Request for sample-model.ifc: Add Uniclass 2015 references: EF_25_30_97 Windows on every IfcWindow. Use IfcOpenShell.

First a look at what the model holds.

```python
import ifcopenshell

model = ifcopenshell.open("sample-model.ifc")
print(model.schema)
print("classifications:", [c.Name for c in model.by_type("IfcClassification")])
for ifc_class in ("IfcDoor", "IfcRoof", "IfcStair", "IfcWall", "IfcWindow"):
    print(ifc_class, len(model.by_type(ifc_class)))
```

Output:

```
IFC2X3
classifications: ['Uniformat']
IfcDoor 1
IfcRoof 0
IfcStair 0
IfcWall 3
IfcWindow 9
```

```python
import ifcopenshell
import ifcopenshell.api.classification

model = ifcopenshell.open("sample-model.ifc")

# IFC2X3 requires Source and Edition and has no link from the project to the system.
system = model.create_entity("IfcClassification", Source="NBS", Edition="2015", Name="Uniclass 2015")

codes = {
    "IfcWindow": ("EF_25_30_97", "Windows"),
}
for ifc_class, (code, name) in codes.items():
    products = model.by_type(ifc_class)
    ifcopenshell.api.classification.add_reference(
        model, products=products, classification=system, identification=code, name=name
    )
    print(code, len(products))

model.write("sample-model_updated.ifc")
```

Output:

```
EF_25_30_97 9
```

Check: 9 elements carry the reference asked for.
